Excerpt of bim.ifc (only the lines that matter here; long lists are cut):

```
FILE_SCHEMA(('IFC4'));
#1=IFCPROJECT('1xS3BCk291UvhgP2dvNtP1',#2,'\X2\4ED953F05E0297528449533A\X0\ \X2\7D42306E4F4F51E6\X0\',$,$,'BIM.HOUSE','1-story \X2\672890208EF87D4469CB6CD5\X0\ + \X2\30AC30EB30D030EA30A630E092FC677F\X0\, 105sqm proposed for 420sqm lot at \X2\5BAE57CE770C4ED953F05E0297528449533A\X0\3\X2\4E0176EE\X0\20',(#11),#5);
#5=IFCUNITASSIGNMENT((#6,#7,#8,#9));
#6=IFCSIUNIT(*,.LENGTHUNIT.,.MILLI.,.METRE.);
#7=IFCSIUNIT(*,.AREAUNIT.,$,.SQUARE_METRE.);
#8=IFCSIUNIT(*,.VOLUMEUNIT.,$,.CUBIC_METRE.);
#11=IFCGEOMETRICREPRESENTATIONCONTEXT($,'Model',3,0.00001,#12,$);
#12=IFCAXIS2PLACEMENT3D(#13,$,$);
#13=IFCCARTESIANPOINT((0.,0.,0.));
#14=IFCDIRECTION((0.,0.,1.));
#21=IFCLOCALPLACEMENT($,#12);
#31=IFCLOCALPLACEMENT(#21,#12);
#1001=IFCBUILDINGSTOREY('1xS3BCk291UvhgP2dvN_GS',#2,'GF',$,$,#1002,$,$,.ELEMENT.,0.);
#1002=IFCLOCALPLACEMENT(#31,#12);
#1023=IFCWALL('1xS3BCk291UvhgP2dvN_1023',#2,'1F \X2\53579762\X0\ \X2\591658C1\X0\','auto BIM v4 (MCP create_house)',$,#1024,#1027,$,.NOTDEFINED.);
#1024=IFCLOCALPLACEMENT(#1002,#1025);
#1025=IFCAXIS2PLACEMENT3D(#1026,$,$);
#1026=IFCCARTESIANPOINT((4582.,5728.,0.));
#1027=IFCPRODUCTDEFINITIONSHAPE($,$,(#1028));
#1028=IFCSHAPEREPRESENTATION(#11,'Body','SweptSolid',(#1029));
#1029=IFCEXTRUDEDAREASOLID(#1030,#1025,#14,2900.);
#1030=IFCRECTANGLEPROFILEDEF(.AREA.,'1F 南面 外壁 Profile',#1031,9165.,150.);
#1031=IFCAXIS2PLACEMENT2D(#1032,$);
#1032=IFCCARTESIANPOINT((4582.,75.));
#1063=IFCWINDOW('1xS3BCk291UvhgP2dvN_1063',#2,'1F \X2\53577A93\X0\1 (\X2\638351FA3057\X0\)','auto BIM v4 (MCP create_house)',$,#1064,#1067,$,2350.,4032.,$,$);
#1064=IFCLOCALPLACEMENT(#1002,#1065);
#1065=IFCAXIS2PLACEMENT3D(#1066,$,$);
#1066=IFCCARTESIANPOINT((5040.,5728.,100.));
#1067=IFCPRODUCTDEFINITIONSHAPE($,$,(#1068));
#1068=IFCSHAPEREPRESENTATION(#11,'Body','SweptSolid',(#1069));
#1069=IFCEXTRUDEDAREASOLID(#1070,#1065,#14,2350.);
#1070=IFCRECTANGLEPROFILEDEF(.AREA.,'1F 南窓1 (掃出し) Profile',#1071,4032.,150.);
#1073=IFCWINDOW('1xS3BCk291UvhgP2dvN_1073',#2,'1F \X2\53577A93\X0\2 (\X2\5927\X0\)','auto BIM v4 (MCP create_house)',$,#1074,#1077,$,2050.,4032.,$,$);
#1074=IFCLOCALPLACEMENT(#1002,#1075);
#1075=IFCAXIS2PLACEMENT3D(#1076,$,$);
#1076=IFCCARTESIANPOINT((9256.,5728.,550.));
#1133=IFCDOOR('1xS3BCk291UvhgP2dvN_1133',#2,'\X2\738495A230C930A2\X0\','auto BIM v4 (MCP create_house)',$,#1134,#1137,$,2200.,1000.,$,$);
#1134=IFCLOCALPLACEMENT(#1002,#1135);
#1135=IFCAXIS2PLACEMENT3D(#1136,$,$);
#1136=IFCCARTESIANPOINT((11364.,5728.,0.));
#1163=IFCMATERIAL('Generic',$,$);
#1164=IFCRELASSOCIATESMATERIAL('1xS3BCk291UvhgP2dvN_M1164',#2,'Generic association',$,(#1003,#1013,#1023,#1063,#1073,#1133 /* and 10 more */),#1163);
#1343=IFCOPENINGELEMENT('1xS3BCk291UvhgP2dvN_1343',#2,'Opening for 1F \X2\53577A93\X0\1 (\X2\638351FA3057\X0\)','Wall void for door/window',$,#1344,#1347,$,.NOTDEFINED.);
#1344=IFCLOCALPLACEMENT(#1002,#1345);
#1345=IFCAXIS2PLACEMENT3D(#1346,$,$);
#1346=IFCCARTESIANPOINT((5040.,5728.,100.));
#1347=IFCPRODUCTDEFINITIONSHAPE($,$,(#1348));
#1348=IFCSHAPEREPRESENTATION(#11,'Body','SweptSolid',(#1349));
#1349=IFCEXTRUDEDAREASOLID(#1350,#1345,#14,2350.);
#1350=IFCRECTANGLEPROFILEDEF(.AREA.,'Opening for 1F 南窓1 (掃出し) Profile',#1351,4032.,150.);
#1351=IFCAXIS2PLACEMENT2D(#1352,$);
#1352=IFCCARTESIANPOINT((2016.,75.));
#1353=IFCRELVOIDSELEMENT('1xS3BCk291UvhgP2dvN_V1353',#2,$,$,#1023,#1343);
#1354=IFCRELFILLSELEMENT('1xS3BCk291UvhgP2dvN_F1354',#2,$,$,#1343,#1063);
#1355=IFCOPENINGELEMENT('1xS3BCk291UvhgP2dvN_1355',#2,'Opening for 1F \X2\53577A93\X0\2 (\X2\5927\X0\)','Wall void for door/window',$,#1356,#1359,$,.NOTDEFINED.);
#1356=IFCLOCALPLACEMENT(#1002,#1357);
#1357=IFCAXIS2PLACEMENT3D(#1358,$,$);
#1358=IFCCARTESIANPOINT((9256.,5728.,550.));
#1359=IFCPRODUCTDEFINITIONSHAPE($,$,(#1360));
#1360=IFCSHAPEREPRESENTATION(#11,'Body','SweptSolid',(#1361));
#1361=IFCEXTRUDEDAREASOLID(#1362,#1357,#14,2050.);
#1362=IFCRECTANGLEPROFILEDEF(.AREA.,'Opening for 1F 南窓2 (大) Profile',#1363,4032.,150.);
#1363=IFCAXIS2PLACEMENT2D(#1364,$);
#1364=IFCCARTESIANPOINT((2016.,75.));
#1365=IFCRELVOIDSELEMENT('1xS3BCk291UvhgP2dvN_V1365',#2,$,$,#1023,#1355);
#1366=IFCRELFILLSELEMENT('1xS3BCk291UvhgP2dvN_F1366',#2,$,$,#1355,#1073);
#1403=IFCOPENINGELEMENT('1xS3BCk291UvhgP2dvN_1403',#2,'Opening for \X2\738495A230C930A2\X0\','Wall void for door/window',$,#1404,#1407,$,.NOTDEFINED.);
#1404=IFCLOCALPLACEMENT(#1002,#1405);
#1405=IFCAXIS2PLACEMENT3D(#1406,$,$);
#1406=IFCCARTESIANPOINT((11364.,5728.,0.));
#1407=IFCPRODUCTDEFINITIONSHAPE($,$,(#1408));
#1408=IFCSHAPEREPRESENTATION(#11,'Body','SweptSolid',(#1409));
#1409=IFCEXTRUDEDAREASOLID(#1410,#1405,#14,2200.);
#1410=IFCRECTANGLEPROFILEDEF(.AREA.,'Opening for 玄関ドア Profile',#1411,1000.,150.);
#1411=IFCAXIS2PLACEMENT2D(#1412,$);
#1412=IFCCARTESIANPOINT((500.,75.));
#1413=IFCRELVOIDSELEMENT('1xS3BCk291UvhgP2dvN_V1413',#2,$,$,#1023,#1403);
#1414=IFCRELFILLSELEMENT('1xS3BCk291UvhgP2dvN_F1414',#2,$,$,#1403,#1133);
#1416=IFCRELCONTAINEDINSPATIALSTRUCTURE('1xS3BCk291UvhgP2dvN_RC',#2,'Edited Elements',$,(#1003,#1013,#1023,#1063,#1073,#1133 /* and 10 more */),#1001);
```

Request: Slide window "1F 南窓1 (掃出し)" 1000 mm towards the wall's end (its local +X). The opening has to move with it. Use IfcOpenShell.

```python
import ifcopenshell
import ifcopenshell.api.geometry
import ifcopenshell.util.placement
import ifcopenshell.util.unit

model = ifcopenshell.open("bim.ifc")
unit_scale = ifcopenshell.util.unit.calculate_unit_scale(model)

window = model.by_guid("1xS3BCk291UvhgP2dvN_1063")
opening = window.FillsVoids[0].RelatingOpeningElement
wall = opening.VoidsElements[0].RelatingBuildingElement

wall_matrix = ifcopenshell.util.placement.get_local_placement(wall.ObjectPlacement)
shift = wall_matrix[:3, 0] * 1 / unit_scale
before = ifcopenshell.util.placement.get_local_placement(window.ObjectPlacement)[:3, 3].copy()

# The window is not placed relative to its opening, so move both.
for product in (opening, window):
    matrix = ifcopenshell.util.placement.get_local_placement(product.ObjectPlacement)
    matrix[:3, 3] += shift
    ifcopenshell.api.geometry.edit_object_placement(model, product=product, matrix=matrix, is_si=False)

after = ifcopenshell.util.placement.get_local_placement(window.ObjectPlacement)[:3, 3]
print("window moved by", (after - before).round(3) + 0.0)

model.write("bim_edited.ifc")
```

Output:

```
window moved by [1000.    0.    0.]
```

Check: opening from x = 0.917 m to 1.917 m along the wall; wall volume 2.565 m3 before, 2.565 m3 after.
